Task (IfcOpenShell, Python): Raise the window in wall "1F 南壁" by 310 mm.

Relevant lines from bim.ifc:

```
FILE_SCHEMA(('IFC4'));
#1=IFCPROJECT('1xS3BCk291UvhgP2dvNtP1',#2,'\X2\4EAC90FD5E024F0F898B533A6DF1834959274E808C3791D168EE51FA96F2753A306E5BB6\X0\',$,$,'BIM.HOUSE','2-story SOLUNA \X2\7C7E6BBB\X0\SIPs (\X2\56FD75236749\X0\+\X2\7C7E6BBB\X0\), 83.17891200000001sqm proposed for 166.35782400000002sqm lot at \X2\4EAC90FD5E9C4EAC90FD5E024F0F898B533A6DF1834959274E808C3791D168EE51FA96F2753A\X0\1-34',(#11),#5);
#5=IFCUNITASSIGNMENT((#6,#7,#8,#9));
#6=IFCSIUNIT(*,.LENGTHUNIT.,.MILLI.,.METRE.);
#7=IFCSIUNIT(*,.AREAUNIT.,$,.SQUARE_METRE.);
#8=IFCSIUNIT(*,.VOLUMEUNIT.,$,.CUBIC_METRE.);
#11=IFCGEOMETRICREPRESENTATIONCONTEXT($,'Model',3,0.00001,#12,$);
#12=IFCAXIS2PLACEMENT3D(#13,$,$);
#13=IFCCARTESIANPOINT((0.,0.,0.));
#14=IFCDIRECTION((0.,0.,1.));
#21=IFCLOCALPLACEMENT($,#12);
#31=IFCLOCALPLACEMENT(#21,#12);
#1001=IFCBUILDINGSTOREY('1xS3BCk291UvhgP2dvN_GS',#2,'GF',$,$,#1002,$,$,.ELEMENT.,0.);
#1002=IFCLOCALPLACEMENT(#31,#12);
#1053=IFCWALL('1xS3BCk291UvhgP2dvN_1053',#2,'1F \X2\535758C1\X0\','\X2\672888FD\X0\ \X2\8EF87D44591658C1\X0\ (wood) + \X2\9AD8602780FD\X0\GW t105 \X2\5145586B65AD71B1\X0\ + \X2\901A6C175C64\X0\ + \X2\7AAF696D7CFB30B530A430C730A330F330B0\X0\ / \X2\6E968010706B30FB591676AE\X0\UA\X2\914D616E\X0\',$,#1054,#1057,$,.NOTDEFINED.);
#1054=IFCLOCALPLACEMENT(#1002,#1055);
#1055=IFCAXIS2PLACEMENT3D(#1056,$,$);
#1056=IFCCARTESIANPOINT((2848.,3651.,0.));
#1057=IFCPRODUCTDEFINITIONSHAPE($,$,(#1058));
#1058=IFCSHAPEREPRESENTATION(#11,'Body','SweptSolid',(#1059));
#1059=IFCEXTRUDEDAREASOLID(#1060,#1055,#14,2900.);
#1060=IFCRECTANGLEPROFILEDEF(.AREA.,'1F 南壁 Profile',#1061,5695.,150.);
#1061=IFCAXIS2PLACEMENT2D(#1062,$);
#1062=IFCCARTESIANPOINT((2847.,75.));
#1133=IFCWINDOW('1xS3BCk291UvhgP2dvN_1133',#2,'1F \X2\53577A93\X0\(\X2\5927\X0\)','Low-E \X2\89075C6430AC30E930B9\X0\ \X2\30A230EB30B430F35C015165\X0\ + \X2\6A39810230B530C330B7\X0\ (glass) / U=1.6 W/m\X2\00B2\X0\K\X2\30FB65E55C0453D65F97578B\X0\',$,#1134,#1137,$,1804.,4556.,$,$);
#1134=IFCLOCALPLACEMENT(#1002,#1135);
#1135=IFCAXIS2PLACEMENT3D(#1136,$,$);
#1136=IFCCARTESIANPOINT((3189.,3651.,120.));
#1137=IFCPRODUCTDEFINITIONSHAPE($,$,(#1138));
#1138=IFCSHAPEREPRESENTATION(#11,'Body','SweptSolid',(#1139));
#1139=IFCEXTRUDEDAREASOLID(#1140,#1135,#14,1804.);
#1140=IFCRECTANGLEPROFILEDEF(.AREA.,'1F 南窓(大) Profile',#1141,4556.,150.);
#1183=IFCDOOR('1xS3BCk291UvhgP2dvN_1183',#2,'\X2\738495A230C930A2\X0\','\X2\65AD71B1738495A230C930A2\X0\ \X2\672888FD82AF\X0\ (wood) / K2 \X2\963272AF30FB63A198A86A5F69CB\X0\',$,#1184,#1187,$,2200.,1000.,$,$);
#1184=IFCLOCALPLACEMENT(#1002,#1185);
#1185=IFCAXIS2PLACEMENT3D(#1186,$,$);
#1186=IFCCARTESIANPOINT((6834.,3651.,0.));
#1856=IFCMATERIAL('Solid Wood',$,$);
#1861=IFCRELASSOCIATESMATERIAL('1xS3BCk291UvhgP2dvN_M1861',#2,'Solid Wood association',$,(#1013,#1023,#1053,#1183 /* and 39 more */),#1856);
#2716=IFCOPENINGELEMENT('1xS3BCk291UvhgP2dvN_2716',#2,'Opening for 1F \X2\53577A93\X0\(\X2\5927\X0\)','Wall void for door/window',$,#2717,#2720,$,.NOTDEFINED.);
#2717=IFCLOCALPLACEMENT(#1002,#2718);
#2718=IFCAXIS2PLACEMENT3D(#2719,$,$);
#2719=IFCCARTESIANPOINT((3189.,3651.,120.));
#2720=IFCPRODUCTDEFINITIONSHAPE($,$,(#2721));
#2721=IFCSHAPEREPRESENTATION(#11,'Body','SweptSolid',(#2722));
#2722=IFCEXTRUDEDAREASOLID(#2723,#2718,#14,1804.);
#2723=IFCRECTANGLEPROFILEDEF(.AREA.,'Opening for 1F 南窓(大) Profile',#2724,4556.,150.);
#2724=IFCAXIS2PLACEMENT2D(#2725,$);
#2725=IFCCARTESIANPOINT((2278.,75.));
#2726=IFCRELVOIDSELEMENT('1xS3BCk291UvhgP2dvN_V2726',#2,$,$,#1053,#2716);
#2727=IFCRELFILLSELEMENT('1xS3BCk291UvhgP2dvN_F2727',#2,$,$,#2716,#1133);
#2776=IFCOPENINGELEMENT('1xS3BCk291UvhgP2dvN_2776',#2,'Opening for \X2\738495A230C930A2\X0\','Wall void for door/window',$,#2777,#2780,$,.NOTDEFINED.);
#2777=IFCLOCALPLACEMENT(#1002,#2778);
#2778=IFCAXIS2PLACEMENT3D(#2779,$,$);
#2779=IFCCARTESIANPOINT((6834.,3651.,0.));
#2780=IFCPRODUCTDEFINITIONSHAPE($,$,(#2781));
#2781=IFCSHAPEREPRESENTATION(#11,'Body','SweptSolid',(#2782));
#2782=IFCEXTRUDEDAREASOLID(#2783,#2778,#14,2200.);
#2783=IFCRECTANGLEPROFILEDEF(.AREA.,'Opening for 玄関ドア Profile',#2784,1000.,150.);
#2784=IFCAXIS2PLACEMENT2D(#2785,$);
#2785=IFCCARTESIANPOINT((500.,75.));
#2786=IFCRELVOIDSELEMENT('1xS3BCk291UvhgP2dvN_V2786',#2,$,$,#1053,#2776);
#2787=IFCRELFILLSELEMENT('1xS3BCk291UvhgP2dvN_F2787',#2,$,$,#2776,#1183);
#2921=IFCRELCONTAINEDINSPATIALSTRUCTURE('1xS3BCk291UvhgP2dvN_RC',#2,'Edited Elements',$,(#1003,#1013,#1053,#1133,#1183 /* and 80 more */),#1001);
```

```python
import numpy as np
import ifcopenshell
import ifcopenshell.api.geometry
import ifcopenshell.util.placement
import ifcopenshell.util.unit

model = ifcopenshell.open("bim.ifc")
unit_scale = ifcopenshell.util.unit.calculate_unit_scale(model)

window = model.by_id(1133)
opening = window.FillsVoids[0].RelatingOpeningElement
dz = 0.31 / unit_scale

shift = np.array([0.0, 0.0, dz])
# The window is not placed relative to its opening, so move both.
for product in (opening, window):
    matrix = ifcopenshell.util.placement.get_local_placement(product.ObjectPlacement)
    matrix[:3, 3] += shift
    ifcopenshell.api.geometry.edit_object_placement(model, product=product, matrix=matrix, is_si=False)

print(f"moved by {dz * unit_scale:+.3f} m")

model.write("bim_rev.ifc")
```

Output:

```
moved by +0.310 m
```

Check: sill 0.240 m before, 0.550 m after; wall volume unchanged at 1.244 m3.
